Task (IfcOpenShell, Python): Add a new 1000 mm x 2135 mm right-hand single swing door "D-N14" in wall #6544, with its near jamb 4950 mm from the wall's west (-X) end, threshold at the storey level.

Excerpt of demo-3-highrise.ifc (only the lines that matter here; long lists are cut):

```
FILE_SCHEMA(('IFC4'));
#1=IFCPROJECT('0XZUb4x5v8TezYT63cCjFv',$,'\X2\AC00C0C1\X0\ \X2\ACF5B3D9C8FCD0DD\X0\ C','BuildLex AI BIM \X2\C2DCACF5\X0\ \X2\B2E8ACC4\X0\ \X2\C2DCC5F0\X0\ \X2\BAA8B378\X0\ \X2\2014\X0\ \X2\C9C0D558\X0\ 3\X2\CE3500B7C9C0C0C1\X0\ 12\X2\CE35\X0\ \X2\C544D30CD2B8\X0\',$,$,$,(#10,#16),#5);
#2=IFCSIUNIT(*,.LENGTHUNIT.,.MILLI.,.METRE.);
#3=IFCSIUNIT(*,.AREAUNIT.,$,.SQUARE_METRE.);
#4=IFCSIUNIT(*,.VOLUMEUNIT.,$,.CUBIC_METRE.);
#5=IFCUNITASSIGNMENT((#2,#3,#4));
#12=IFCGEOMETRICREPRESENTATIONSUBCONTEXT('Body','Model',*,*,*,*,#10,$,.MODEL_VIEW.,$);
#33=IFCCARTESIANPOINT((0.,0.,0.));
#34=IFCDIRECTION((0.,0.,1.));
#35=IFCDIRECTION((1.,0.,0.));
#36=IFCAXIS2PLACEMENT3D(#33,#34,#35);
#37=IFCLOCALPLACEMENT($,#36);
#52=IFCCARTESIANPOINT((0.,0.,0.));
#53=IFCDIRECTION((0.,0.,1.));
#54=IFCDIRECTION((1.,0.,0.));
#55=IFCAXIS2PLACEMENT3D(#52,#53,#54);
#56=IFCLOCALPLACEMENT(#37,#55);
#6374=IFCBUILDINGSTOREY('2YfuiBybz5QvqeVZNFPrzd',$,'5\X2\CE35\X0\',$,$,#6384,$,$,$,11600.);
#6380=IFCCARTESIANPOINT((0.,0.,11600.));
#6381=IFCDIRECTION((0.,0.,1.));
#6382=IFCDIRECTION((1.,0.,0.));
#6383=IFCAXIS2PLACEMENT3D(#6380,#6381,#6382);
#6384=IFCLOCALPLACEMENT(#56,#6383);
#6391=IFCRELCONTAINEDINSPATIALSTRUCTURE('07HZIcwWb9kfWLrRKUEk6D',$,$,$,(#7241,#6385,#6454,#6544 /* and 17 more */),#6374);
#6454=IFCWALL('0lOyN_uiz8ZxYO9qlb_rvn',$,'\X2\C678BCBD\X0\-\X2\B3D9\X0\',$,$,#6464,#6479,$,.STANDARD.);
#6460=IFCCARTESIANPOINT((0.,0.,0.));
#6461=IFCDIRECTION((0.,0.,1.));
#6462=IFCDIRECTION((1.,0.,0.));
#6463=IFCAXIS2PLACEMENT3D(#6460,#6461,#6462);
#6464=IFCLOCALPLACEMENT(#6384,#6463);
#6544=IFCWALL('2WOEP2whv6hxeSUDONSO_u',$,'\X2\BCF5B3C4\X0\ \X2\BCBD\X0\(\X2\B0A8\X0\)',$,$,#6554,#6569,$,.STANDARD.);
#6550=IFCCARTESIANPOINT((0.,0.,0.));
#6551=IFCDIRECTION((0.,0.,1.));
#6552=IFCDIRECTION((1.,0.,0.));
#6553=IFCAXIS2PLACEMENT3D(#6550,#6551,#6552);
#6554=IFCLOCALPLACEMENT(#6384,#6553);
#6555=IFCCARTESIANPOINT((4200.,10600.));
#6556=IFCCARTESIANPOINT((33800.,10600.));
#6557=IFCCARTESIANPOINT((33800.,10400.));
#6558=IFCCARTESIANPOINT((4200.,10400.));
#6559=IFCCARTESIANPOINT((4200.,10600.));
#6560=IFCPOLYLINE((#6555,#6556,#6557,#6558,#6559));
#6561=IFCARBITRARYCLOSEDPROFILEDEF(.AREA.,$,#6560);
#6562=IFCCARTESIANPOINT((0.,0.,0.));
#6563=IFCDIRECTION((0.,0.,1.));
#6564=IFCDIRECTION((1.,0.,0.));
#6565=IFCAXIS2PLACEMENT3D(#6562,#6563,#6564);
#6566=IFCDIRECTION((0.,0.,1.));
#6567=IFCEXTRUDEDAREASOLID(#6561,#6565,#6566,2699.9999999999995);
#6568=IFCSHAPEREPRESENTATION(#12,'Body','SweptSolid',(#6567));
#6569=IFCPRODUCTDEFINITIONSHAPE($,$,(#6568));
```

```python
import numpy as np
import ifcopenshell
import ifcopenshell.api.feature
import ifcopenshell.api.geometry
import ifcopenshell.api.root
import ifcopenshell.api.spatial
import ifcopenshell.geom
import ifcopenshell.util.element
import ifcopenshell.util.placement
import ifcopenshell.util.representation
import ifcopenshell.util.shape
import ifcopenshell.util.unit

model = ifcopenshell.open("demo-3-highrise.ifc")
unit_scale = ifcopenshell.util.unit.calculate_unit_scale(model)
settings = ifcopenshell.geom.settings()


def volume(element):
    """Net volume in cubic metres, openings subtracted."""
    shape = ifcopenshell.geom.create_shape(settings, element)
    return ifcopenshell.util.shape.get_volume(shape.geometry)


wall = model.by_guid("2WOEP2whv6hxeSUDONSO_u")
storey = ifcopenshell.util.element.get_container(wall, ifc_class="IfcBuildingStorey")
context = ifcopenshell.util.representation.get_context(model, "Model", "Body", "MODEL_VIEW")
before = volume(wall)

width, height, from_end, sill = 1, 2.135, 4.95, 0.0  # metres

# The wall runs along its own X axis, and the end named is its -X end.
wall_shape = ifcopenshell.geom.create_shape(settings, wall)
x, y, z = ifcopenshell.util.shape.get_vertices(wall_shape.geometry).T
start = x.min() + from_end
face, thickness = float(y.min()), float(y.max() - y.min())
wall_matrix = ifcopenshell.util.placement.get_local_placement(wall.ObjectPlacement)
level = ifcopenshell.util.placement.get_local_placement(storey.ObjectPlacement)[2, 3]


def in_wall(x, y):
    """Placement at x, y metres in the wall's axes, at sill height."""
    matrix = wall_matrix.copy()
    matrix[:, 3] = wall_matrix @ np.array([x / unit_scale, y / unit_scale, 0.0, 1.0])
    matrix[2, 3] = level + sill / unit_scale
    return matrix


# Opening: a box that overshoots both wall faces by 50 mm.
opening = ifcopenshell.api.root.create_entity(model, ifc_class="IfcOpeningElement", predefined_type="OPENING")
box = ifcopenshell.api.geometry.add_wall_representation(
    model, context=context, length=width, height=height, thickness=thickness + 0.1
)
ifcopenshell.api.geometry.assign_representation(model, product=opening, representation=box)
ifcopenshell.api.geometry.edit_object_placement(model, product=opening, matrix=in_wall(start, face - 0.05), is_si=False)
ifcopenshell.api.feature.add_feature(model, feature=opening, element=wall)

door = ifcopenshell.api.root.create_entity(model, ifc_class="IfcDoor", name="D-N14", predefined_type="DOOR")
door.OverallWidth, door.OverallHeight = width / unit_scale, height / unit_scale
door.OperationType = "SINGLE_SWING_RIGHT"
body = ifcopenshell.api.geometry.add_door_representation(
    model,
    context=context,
    overall_width=door.OverallWidth,
    overall_height=door.OverallHeight,
    operation_type="SINGLE_SWING_RIGHT",
    lining_properties={"LiningDepth": thickness / unit_scale, "ThresholdDepth": thickness / unit_scale},
)
ifcopenshell.api.geometry.assign_representation(model, product=door, representation=body)
ifcopenshell.api.spatial.assign_container(model, products=[door], relating_structure=storey)
ifcopenshell.api.feature.add_filling(model, opening=opening, element=door)

# The lining spans the wall, so the door starts at the wall face.
ifcopenshell.api.geometry.edit_object_placement(model, product=door, matrix=in_wall(start, face), is_si=False)

after = volume(wall)

print(f"wall volume {before:.3f} -> {after:.3f} m3")

model.write("demo-3-highrise-out.ifc")
```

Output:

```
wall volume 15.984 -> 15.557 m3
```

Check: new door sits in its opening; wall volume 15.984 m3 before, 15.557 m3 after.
